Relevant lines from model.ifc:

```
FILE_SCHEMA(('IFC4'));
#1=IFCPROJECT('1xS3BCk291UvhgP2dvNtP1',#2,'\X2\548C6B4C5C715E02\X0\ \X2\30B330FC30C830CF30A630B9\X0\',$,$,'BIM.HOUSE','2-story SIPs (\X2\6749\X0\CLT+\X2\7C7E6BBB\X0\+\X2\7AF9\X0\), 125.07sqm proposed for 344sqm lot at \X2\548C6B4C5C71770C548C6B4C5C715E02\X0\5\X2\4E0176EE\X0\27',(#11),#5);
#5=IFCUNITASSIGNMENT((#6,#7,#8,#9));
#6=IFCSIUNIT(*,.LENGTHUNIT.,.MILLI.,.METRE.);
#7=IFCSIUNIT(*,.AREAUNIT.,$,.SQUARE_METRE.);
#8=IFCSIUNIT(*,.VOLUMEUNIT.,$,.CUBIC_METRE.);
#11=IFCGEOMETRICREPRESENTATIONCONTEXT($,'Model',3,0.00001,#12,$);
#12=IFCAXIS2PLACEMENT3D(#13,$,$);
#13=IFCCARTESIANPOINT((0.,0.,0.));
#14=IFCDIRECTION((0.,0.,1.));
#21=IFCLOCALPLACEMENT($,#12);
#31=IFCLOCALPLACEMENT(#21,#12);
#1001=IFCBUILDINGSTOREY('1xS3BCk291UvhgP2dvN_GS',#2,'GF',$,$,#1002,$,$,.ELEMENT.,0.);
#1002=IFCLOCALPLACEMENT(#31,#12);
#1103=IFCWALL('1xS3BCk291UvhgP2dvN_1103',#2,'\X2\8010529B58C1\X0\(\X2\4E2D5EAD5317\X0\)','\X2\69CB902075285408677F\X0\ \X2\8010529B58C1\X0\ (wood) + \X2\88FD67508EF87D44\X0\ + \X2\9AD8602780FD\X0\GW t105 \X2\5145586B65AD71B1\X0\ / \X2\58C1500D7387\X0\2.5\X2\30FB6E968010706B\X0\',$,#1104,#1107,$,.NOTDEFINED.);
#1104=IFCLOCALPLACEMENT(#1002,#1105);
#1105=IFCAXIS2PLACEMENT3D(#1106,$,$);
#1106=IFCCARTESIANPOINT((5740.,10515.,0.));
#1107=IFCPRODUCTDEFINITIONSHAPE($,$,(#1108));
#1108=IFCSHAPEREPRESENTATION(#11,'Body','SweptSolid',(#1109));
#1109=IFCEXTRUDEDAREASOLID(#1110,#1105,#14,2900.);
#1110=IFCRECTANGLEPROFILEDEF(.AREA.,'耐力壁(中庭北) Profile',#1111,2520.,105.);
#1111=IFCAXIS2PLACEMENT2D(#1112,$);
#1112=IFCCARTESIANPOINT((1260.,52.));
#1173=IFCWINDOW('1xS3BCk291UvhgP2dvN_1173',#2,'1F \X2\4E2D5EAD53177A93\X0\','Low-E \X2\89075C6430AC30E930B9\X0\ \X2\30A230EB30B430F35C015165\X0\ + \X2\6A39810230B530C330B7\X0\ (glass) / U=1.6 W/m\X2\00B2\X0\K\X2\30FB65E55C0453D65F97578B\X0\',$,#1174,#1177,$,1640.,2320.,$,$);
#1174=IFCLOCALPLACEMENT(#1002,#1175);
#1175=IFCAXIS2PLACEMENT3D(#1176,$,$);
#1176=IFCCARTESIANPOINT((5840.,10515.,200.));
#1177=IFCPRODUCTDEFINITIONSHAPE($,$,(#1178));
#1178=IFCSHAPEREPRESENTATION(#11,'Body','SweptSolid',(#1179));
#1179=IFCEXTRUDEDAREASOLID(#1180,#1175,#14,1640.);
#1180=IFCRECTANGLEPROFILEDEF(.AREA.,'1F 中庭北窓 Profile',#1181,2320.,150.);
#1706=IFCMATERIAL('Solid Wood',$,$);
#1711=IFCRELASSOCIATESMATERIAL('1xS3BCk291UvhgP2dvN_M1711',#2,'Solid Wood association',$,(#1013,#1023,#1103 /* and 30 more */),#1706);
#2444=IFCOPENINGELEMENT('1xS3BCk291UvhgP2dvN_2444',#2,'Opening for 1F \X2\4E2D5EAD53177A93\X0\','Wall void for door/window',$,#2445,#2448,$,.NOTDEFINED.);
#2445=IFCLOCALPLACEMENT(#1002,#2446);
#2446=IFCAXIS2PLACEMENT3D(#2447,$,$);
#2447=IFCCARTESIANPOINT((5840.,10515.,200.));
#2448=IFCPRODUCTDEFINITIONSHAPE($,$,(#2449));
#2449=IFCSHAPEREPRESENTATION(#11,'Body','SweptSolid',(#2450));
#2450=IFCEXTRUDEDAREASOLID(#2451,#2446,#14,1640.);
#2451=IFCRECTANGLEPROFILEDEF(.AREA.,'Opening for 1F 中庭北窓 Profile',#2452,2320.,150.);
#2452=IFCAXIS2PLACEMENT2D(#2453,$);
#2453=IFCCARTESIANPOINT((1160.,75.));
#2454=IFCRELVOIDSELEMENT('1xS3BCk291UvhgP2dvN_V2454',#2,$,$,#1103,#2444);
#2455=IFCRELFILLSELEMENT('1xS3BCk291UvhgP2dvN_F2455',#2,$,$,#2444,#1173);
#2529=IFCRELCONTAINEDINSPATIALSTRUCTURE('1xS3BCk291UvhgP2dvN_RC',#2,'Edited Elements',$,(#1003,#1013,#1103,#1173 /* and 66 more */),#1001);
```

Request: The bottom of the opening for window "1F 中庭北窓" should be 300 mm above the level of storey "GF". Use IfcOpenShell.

```python
import numpy as np
import ifcopenshell
import ifcopenshell.api.geometry
import ifcopenshell.geom
import ifcopenshell.util.element
import ifcopenshell.util.placement
import ifcopenshell.util.shape
import ifcopenshell.util.unit

model = ifcopenshell.open("model.ifc")
unit_scale = ifcopenshell.util.unit.calculate_unit_scale(model)

window = model.by_guid("1xS3BCk291UvhgP2dvN_1173")
opening = window.FillsVoids[0].RelatingOpeningElement
storey = ifcopenshell.util.element.get_container(window, ifc_class="IfcBuildingStorey")
level = ifcopenshell.util.placement.get_local_placement(storey.ObjectPlacement)[2, 3]

# The opening's origin need not be at the sill, so measure its lowest point.
shape = ifcopenshell.geom.create_shape(ifcopenshell.geom.settings(), opening)
bottom = ifcopenshell.util.shape.get_shape_bottom_elevation(shape, shape.geometry) / unit_scale
dz = level + 0.3 / unit_scale - bottom

shift = np.array([0.0, 0.0, dz])
# The window is not placed relative to its opening, so move both.
for product in (opening, window):
    matrix = ifcopenshell.util.placement.get_local_placement(product.ObjectPlacement)
    matrix[:3, 3] += shift
    ifcopenshell.api.geometry.edit_object_placement(model, product=product, matrix=matrix, is_si=False)

print(f"moved by {dz * unit_scale:+.3f} m")

model.write("model_updated.ifc")
```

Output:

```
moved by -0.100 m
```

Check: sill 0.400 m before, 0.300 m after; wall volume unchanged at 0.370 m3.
